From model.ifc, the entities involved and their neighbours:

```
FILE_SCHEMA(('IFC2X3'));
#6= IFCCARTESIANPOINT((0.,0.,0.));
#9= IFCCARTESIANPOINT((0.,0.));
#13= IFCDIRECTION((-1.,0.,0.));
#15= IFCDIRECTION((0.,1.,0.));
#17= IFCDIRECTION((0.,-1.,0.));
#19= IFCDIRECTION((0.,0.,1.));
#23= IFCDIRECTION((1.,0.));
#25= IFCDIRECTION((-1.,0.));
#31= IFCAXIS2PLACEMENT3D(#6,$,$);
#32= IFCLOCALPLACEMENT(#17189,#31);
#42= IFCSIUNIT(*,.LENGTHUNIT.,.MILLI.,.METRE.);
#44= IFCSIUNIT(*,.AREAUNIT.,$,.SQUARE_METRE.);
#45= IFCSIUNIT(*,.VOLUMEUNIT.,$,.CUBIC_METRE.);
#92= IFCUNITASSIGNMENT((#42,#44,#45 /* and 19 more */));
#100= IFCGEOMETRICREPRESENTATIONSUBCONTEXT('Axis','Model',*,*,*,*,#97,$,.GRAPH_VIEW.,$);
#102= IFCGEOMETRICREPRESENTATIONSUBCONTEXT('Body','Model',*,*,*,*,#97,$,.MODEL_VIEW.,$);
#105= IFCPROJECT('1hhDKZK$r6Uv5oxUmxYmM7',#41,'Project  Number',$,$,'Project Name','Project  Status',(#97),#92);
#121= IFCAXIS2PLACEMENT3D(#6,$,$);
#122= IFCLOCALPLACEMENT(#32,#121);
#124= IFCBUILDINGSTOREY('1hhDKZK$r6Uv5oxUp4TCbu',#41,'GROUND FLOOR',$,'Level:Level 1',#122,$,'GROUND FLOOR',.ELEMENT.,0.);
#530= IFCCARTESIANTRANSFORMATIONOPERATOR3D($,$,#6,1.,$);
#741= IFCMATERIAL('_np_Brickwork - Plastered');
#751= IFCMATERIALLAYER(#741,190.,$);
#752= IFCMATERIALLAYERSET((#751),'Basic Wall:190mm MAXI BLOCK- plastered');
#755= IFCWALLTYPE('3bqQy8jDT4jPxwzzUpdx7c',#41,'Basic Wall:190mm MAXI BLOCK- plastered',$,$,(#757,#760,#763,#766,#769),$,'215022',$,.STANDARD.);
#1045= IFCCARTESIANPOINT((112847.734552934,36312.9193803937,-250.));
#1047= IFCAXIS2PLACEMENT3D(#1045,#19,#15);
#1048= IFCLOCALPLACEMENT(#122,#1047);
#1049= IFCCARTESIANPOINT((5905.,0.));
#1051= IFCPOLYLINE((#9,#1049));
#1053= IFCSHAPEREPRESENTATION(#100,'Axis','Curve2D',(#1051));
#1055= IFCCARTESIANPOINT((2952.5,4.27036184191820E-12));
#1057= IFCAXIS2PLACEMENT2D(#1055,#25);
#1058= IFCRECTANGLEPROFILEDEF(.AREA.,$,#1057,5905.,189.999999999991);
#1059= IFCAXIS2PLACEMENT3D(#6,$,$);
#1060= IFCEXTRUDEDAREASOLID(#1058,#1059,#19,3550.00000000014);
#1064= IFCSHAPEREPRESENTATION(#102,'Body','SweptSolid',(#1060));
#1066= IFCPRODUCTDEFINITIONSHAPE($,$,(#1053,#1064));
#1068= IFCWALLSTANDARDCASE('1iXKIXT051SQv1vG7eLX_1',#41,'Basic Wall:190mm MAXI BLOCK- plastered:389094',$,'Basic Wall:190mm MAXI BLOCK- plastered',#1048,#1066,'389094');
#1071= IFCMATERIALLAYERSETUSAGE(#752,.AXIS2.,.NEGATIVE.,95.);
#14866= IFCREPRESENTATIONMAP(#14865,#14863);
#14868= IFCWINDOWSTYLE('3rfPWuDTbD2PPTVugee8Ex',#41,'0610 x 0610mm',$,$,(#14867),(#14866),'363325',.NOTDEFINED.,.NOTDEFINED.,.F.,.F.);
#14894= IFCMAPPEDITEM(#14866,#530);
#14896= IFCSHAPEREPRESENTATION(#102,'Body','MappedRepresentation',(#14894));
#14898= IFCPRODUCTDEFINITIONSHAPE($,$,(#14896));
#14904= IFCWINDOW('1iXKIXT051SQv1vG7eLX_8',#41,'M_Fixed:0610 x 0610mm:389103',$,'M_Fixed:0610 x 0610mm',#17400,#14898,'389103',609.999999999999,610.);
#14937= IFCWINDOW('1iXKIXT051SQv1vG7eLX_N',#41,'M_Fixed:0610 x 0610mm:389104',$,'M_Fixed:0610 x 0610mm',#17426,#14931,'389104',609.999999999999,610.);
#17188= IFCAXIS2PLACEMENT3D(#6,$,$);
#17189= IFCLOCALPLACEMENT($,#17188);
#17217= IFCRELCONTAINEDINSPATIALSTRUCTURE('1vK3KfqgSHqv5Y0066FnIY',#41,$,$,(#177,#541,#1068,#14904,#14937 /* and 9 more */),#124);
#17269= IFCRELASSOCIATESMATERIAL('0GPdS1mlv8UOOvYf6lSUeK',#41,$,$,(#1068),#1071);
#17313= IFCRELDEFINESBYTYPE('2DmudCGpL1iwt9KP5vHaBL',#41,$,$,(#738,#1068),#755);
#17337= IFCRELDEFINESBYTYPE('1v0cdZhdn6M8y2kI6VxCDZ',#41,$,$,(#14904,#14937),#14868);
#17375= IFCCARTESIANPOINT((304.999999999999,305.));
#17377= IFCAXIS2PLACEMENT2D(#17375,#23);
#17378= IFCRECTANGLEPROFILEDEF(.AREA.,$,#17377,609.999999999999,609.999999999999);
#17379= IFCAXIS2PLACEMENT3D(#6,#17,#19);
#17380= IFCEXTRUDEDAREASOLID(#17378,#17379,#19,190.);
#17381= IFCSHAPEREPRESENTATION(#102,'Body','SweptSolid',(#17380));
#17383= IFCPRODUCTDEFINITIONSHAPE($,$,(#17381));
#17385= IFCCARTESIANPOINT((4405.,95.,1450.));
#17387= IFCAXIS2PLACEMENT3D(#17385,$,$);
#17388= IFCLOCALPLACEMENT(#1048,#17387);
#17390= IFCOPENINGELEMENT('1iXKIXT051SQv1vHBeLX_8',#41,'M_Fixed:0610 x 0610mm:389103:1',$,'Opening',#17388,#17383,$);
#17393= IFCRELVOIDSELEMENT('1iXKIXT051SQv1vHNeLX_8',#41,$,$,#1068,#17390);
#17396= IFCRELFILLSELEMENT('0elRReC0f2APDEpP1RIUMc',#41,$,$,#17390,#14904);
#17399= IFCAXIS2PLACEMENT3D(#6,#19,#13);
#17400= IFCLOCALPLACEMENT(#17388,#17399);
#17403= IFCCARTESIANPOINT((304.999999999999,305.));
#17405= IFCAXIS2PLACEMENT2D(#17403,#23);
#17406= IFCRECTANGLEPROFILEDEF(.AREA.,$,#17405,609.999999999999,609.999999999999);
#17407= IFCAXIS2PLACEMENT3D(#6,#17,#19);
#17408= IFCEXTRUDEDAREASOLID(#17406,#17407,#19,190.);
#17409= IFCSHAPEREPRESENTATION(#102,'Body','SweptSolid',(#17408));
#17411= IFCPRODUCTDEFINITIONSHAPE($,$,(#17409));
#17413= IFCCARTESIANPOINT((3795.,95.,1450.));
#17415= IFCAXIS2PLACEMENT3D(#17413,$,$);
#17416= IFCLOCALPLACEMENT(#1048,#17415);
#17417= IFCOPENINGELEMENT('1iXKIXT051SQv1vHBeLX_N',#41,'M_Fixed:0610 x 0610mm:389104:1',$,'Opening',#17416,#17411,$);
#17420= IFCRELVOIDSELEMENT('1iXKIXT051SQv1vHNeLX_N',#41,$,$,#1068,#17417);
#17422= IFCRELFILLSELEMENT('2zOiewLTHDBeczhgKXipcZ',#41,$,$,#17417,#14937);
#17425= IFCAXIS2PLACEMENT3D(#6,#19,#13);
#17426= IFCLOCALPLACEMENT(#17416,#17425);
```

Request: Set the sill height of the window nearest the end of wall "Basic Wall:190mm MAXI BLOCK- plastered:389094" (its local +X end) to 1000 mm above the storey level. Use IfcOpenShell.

```python
import numpy as np
import ifcopenshell
import ifcopenshell.api.geometry
import ifcopenshell.geom
import ifcopenshell.util.element
import ifcopenshell.util.placement
import ifcopenshell.util.shape
import ifcopenshell.util.unit

model = ifcopenshell.open("model.ifc")
unit_scale = ifcopenshell.util.unit.calculate_unit_scale(model)

window = model.by_guid("1iXKIXT051SQv1vG7eLX_8")
opening = window.FillsVoids[0].RelatingOpeningElement
storey = ifcopenshell.util.element.get_container(window, ifc_class="IfcBuildingStorey")
level = ifcopenshell.util.placement.get_local_placement(storey.ObjectPlacement)[2, 3]

# The opening's origin need not be at the sill, so measure its lowest point.
shape = ifcopenshell.geom.create_shape(ifcopenshell.geom.settings(), opening)
bottom = ifcopenshell.util.shape.get_shape_bottom_elevation(shape, shape.geometry) / unit_scale
dz = level + 1 / unit_scale - bottom

shift = np.array([0.0, 0.0, dz])
# The window is placed relative to its opening, so it follows when the opening moves.
matrix = ifcopenshell.util.placement.get_local_placement(opening.ObjectPlacement)
matrix[:3, 3] += shift
ifcopenshell.api.geometry.edit_object_placement(
    model, product=opening, matrix=matrix, is_si=False, should_transform_children=True
)

print(f"moved by {dz * unit_scale:+.3f} m")

model.write("model_rev.ifc")
```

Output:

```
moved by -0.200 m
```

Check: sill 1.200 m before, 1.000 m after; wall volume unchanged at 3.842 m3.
